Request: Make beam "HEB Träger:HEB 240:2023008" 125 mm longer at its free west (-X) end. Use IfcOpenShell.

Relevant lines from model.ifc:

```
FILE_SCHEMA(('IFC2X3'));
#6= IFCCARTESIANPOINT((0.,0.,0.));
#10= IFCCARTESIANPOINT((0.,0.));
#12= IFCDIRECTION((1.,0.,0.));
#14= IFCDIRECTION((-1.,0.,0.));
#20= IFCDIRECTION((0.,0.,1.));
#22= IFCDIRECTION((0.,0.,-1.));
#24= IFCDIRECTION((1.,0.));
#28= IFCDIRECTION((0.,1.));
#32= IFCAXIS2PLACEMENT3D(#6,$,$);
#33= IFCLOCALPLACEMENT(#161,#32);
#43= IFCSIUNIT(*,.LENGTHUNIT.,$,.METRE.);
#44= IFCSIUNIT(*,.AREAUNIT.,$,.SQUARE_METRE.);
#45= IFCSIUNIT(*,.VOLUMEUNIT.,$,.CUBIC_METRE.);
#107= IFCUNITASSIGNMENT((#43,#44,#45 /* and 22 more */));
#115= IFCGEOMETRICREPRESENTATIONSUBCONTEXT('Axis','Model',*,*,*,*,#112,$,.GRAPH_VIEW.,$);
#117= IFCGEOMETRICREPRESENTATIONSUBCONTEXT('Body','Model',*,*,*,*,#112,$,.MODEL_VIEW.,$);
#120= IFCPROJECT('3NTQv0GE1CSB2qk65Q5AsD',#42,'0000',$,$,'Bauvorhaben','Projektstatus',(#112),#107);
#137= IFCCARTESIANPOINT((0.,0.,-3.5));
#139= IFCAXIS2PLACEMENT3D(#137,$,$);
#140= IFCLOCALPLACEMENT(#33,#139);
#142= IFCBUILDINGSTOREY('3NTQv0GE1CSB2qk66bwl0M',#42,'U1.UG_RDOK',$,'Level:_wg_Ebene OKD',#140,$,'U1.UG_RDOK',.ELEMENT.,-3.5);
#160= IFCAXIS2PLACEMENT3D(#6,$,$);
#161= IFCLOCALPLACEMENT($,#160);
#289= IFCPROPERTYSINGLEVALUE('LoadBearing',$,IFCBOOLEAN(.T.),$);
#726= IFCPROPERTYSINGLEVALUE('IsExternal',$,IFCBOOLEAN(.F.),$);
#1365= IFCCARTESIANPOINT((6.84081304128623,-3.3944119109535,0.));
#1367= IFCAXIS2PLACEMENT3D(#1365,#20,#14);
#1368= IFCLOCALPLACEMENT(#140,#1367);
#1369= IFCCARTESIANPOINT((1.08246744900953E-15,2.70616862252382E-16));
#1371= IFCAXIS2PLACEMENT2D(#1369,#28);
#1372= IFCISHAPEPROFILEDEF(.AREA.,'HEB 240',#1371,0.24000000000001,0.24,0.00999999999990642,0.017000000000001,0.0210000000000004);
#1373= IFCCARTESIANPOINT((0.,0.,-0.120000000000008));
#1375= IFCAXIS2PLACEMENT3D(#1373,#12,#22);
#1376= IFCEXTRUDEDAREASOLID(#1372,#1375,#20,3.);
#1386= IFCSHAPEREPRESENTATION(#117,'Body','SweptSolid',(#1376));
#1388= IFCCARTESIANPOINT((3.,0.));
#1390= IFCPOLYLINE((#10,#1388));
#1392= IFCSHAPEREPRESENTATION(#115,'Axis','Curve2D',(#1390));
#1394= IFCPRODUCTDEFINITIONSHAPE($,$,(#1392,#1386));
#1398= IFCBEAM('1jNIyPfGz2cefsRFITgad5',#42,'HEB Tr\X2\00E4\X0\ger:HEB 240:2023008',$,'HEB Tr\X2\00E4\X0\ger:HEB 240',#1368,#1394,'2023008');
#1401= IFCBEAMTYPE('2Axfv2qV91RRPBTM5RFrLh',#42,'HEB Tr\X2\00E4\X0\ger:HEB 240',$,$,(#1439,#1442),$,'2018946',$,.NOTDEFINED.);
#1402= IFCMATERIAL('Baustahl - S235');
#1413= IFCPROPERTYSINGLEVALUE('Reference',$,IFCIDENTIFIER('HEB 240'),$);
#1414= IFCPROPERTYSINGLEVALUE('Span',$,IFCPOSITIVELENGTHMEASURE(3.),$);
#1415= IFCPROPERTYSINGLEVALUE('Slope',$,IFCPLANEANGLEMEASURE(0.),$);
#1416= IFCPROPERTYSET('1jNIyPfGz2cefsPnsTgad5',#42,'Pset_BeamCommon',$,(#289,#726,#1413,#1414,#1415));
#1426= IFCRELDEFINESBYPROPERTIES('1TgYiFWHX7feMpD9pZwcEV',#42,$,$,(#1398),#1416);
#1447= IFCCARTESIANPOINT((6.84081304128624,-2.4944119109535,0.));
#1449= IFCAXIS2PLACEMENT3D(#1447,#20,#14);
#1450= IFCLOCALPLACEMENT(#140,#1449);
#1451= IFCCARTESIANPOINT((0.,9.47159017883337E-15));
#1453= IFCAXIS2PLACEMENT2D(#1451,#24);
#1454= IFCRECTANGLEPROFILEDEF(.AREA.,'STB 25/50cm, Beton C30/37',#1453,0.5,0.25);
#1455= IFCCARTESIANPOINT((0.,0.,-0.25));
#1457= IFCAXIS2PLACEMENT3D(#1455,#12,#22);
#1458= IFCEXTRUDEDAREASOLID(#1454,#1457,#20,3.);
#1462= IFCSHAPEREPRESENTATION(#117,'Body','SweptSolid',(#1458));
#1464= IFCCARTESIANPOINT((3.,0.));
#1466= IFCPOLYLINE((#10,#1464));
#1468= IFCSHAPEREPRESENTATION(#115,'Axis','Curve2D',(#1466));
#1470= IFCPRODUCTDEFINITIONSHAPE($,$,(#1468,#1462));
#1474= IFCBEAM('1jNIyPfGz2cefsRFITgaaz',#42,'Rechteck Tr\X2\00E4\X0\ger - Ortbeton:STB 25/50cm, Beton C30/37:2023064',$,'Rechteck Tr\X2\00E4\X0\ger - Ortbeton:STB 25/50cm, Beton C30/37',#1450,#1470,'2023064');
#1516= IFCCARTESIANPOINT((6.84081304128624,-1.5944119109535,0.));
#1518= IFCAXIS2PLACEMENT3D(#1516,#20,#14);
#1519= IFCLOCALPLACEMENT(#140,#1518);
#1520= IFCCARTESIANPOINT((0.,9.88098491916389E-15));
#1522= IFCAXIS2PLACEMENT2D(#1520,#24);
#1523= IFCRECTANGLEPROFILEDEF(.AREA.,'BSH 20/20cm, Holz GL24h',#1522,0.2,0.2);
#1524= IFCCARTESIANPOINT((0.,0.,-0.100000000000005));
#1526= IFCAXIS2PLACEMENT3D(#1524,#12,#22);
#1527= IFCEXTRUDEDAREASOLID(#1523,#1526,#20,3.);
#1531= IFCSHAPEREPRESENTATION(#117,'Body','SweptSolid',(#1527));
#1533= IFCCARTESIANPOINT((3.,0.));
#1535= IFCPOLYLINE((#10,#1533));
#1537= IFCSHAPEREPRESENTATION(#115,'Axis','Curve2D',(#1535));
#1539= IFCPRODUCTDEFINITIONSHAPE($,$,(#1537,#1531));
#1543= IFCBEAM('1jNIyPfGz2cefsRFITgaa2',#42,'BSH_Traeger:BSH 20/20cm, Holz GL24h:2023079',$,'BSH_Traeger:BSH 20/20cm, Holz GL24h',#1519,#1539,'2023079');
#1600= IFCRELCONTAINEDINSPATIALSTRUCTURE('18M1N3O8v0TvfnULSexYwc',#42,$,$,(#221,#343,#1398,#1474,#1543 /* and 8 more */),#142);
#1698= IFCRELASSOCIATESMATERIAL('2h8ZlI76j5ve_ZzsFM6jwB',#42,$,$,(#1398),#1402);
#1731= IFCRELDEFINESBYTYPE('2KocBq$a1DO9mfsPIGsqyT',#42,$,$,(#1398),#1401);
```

```python
import numpy as np
import ifcopenshell
import ifcopenshell.api.pset
import ifcopenshell.util.element
import ifcopenshell.util.representation
import ifcopenshell.util.unit

model = ifcopenshell.open("model.ifc")
unit_scale = ifcopenshell.util.unit.calculate_unit_scale(model)

member = model.by_guid("1jNIyPfGz2cefsRFITgad5")
change = 0.125 / unit_scale

# The extrusion runs towards the end named, so only its depth changes.
body = ifcopenshell.util.representation.get_representation(member, "Model", "Body")
solid = body.Items[0]
old_length = solid.Depth
solid.Depth += change

# Move the axis end point with it.
axis = next(r for r in member.Representation.Representations if r.RepresentationIdentifier == "Axis").Items[0]
start, end = (np.array(p.Coordinates) for p in axis.Points)
end = end + (end - start) / np.linalg.norm(end - start) * change
point = model.createIfcCartesianPoint(end.tolist())
axis.Points = [axis.Points[0], point]

# Update the stored length and volume.
pset = model.by_id(ifcopenshell.util.element.get_pset(member, "Pset_BeamCommon", should_inherit=False)["id"])
ifcopenshell.api.pset.edit_pset(model, pset=pset, properties={
    "Span": model.create_entity("IfcPositiveLengthMeasure", solid.Depth),
})

print(f"length {old_length:g} -> {solid.Depth:g}")

model.write("model_updated.ifc")
```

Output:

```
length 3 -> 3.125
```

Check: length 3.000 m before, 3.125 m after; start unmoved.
